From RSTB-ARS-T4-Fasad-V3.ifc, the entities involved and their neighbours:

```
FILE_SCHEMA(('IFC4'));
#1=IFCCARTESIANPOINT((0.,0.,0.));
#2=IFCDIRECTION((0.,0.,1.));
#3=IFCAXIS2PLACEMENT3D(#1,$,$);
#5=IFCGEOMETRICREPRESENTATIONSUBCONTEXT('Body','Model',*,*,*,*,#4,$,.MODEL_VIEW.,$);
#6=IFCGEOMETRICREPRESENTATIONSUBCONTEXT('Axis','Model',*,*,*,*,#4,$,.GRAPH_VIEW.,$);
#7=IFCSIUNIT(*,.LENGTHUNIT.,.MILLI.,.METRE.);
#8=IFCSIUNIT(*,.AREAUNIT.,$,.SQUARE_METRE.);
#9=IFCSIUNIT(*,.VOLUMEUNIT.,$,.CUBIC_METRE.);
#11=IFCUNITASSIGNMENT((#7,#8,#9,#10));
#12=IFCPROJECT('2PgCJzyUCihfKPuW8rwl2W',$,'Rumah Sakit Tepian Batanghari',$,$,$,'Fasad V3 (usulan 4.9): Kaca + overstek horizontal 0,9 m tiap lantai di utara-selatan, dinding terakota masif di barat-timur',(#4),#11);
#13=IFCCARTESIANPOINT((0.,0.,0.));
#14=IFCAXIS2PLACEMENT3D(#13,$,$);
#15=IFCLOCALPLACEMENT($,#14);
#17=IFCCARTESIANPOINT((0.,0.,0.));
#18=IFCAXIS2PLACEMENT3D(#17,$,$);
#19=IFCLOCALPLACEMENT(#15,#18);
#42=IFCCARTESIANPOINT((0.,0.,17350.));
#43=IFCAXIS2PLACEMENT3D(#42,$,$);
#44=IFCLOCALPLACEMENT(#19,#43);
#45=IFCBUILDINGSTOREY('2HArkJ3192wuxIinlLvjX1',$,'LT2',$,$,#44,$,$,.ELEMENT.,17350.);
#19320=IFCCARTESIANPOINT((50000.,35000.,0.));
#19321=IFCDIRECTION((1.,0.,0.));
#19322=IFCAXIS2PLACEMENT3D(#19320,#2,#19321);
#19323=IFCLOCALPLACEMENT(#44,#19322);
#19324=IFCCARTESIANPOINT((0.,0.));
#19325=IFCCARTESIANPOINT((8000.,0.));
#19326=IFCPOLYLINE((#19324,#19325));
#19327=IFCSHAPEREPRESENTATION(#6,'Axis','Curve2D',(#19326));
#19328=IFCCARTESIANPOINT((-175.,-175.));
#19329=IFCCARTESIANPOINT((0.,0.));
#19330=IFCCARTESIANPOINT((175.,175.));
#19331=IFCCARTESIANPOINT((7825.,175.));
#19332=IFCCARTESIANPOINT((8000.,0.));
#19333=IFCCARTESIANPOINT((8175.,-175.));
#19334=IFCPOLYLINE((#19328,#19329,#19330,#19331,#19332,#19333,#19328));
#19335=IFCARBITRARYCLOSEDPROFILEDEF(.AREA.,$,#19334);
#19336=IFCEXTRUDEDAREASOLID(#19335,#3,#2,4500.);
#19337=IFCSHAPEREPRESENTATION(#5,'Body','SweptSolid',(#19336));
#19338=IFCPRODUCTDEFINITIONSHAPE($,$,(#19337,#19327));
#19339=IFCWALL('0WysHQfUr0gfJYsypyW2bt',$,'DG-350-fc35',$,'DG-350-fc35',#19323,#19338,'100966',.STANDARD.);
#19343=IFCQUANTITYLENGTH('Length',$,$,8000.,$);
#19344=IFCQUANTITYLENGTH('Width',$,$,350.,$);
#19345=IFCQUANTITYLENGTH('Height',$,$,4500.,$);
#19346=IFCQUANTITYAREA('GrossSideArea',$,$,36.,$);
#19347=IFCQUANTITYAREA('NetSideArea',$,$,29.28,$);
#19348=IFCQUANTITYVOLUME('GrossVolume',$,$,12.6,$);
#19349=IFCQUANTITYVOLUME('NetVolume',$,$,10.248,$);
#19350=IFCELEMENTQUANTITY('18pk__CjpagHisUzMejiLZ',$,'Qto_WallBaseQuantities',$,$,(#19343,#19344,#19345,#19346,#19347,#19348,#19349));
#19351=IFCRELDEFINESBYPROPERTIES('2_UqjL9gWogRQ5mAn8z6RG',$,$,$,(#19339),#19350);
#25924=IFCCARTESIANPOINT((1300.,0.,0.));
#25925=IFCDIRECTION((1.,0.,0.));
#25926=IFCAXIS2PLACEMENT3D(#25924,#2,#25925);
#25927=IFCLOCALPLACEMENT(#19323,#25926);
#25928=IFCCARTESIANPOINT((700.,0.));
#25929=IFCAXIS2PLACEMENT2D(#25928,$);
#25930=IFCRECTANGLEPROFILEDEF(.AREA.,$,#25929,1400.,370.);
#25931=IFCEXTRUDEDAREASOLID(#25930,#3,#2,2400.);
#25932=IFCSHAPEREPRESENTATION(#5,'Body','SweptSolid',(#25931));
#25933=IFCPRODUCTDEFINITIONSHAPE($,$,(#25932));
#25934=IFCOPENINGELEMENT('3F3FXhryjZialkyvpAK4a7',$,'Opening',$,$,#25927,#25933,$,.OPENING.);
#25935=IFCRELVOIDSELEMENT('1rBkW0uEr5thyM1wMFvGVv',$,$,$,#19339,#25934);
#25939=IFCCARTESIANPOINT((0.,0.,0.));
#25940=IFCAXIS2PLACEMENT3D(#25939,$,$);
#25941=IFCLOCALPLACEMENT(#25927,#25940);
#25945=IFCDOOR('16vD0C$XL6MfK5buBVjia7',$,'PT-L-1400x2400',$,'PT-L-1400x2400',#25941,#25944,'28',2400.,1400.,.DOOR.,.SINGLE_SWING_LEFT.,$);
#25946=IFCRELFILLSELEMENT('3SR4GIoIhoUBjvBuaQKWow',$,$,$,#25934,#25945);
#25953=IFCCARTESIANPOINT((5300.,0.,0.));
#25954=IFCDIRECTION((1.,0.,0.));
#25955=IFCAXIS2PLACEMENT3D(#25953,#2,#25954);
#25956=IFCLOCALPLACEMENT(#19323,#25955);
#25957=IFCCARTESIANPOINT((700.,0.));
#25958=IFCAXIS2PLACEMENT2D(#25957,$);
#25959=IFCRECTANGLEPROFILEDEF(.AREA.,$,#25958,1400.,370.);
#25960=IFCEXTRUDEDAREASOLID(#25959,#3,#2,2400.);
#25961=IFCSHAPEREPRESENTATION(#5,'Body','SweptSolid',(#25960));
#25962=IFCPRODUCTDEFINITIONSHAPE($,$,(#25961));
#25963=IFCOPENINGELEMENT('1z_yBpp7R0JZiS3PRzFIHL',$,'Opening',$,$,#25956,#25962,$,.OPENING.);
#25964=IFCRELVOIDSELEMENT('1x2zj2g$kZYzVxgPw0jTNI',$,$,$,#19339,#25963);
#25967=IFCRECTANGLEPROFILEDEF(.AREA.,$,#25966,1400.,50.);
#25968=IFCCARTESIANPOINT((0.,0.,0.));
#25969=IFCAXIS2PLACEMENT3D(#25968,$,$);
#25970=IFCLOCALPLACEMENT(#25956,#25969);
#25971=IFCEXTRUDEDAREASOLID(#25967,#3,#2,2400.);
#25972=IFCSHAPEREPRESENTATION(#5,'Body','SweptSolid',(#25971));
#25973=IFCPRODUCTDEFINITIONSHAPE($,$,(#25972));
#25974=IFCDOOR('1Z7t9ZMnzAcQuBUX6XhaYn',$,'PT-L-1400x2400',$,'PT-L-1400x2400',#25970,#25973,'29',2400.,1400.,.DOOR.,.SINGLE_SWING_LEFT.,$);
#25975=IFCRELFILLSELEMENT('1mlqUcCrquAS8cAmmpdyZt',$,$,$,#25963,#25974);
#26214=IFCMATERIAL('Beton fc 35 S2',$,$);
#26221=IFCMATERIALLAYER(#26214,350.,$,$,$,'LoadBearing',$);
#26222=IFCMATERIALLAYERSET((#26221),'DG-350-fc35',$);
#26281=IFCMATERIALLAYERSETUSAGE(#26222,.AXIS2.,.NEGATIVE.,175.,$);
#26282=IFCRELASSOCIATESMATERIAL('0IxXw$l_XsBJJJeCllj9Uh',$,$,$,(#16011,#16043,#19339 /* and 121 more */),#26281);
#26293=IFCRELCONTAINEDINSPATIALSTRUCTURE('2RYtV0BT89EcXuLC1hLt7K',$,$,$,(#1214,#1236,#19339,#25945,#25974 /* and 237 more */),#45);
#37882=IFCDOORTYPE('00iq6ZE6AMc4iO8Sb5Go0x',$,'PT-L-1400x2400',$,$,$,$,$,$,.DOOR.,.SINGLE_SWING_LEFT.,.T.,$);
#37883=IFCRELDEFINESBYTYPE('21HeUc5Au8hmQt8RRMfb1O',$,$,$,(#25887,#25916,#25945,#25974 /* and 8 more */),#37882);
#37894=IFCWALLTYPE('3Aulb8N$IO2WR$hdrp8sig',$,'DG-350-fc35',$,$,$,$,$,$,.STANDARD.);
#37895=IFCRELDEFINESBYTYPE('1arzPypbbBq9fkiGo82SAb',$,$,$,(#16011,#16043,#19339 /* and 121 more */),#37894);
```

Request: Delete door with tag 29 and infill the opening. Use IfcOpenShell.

```python
import ifcopenshell
import ifcopenshell.api.feature
import ifcopenshell.api.pset
import ifcopenshell.api.root
import ifcopenshell.geom
import ifcopenshell.util.element
import ifcopenshell.util.shape
import ifcopenshell.util.unit

model = ifcopenshell.open("RSTB-ARS-T4-Fasad-V3.ifc")
area_scale = ifcopenshell.util.unit.calculate_unit_scale(model, "AREAUNIT")
volume_scale = ifcopenshell.util.unit.calculate_unit_scale(model, "VOLUMEUNIT")
settings = ifcopenshell.geom.settings()


def volume(element):
    """Net volume in cubic metres, openings subtracted."""
    shape = ifcopenshell.geom.create_shape(settings, element)
    return ifcopenshell.util.shape.get_volume(shape.geometry)


door = model.by_guid("1Z7t9ZMnzAcQuBUX6XhaYn")
opening = door.FillsVoids[0].RelatingOpeningElement
wall = opening.VoidsElements[0].RelatingBuildingElement
before = volume(wall)

ifcopenshell.api.root.remove_product(model, product=door)
ifcopenshell.api.feature.remove_feature(model, feature=opening)

after = volume(wall)
thickness = 0.35  # wall thickness in metres

# Update the wall's stored quantities.
qto = model.by_id(ifcopenshell.util.element.get_pset(wall, "Qto_WallBaseQuantities", should_inherit=False)["id"])
ifcopenshell.api.pset.edit_qto(model, qto=qto, properties={
    "NetSideArea": after / thickness / area_scale,
    "NetVolume": after / volume_scale,
})

print(f"wall volume {before:.3f} -> {after:.3f} m3")

model.write("RSTB-ARS-T4-Fasad-V3_edited.ifc")
```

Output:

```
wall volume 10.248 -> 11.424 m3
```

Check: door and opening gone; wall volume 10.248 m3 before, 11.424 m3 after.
